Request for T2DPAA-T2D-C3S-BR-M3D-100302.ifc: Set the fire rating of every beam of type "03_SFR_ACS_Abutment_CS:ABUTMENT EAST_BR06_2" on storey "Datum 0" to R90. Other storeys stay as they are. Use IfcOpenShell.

First a look at what the model holds.

```python
import ifcopenshell
import ifcopenshell.util.element

model = ifcopenshell.open("T2DPAA-T2D-C3S-BR-M3D-100302.ifc")
print(model.schema)
storey = next(s for s in model.by_type("IfcBuildingStorey") if s.Name == "Datum 0")
beams = [e for e in ifcopenshell.util.element.get_decomposition(storey) if e.is_a("IfcBeam")]
seen = {}
for e in beams:
    element_type = ifcopenshell.util.element.get_type(e)
    key = (element_type.Name if element_type != e and element_type else None, ifcopenshell.util.element.get_pset(e, "Pset_BeamCommon", "FireRating"))
    seen[key] = seen.get(key, 0) + 1
for (name, value), count in sorted(seen.items(), key=str):
    print(count, "x", name, "|", value)
```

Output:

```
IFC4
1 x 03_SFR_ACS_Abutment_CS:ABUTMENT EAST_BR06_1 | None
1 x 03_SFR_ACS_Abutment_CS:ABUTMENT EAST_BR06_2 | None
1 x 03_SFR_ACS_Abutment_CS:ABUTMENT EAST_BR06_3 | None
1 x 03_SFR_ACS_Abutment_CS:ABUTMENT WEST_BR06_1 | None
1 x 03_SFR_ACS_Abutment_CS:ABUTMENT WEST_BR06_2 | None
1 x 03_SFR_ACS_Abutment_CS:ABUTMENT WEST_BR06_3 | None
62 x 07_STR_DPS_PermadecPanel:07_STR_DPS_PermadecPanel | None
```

```python
import ifcopenshell
import ifcopenshell.api.pset
import ifcopenshell.util.element

model = ifcopenshell.open("T2DPAA-T2D-C3S-BR-M3D-100302.ifc")

storey = next(s for s in model.by_type("IfcBuildingStorey") if s.Name == "Datum 0")
beams = [e for e in ifcopenshell.util.element.get_decomposition(storey) if e.is_a("IfcBeam")]

count = 0
for e in beams:
    element_type = ifcopenshell.util.element.get_type(e)
    if element_type in (None, e) or element_type.Name != "03_SFR_ACS_Abutment_CS:ABUTMENT EAST_BR06_2":
        continue
    # add_pset returns the element's existing set when there is one.
    pset = ifcopenshell.api.pset.add_pset(model, product=e, name="Pset_BeamCommon")
    ifcopenshell.api.pset.edit_pset(model, pset=pset, properties={"FireRating": "R90"})
    count += 1

print(count, "beams updated")

model.write("T2DPAA-T2D-C3S-BR-M3D-100302-out.ifc")
```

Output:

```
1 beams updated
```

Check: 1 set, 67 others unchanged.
